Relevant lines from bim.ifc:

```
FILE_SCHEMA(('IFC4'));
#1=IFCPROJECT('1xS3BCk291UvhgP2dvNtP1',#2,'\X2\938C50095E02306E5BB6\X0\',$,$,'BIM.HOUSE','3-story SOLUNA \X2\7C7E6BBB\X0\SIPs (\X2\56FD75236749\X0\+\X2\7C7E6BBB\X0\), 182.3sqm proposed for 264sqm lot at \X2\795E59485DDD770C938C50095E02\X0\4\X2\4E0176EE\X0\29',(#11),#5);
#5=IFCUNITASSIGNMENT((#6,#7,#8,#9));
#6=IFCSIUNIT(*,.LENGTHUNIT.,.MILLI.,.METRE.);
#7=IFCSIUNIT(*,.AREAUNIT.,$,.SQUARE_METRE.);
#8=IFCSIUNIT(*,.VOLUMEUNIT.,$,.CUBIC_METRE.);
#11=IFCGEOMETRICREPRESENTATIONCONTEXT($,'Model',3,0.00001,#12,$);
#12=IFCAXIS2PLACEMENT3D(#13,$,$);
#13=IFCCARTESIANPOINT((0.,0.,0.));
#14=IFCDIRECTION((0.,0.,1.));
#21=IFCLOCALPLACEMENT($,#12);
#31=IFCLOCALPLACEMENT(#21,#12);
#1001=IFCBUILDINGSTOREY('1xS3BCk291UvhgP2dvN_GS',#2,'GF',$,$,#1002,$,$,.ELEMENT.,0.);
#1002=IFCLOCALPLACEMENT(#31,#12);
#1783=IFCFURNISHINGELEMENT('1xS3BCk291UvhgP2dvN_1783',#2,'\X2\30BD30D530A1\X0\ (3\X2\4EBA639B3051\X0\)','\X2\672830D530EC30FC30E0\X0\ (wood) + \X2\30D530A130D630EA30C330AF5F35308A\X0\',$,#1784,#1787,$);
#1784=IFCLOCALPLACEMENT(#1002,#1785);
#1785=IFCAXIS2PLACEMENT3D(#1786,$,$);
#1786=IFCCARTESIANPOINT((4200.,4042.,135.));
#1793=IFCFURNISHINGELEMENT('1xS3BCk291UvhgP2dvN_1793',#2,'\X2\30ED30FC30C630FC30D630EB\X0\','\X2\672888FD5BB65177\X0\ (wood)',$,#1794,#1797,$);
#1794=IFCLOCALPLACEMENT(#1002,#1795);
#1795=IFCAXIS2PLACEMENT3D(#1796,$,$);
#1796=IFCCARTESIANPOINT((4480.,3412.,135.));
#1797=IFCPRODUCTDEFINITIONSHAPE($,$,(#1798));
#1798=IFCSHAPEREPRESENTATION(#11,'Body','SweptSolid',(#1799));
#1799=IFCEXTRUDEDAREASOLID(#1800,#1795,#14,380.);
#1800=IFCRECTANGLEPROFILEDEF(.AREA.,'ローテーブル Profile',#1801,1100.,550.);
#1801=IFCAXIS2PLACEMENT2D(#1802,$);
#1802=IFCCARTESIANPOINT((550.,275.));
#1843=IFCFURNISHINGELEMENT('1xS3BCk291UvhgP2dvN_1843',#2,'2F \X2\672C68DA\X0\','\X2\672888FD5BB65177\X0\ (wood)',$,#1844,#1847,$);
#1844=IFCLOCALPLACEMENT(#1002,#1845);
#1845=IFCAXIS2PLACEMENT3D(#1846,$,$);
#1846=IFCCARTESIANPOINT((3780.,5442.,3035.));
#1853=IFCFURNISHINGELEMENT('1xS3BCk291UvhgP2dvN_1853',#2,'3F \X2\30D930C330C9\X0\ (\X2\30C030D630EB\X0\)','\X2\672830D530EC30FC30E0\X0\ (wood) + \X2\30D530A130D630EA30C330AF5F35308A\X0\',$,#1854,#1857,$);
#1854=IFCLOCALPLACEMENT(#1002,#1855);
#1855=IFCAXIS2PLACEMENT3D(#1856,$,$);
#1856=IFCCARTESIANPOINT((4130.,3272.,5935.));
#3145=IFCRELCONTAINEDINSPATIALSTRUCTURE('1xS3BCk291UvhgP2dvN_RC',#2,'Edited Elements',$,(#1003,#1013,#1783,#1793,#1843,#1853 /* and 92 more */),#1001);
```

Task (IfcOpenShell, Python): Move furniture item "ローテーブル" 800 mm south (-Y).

```python
import ifcopenshell
import ifcopenshell.api.geometry
import ifcopenshell.util.placement
import ifcopenshell.util.unit

model = ifcopenshell.open("bim.ifc")
unit_scale = ifcopenshell.util.unit.calculate_unit_scale(model)

item = model.by_id(1793)
matrix = ifcopenshell.util.placement.get_local_placement(item.ObjectPlacement)
matrix[1, 3] -= 0.8 / unit_scale
ifcopenshell.api.geometry.edit_object_placement(model, product=item, matrix=matrix, is_si=False)

print(ifcopenshell.util.placement.get_local_placement(item.ObjectPlacement).round(3) + 0.0)

model.write("bim_updated.ifc")
```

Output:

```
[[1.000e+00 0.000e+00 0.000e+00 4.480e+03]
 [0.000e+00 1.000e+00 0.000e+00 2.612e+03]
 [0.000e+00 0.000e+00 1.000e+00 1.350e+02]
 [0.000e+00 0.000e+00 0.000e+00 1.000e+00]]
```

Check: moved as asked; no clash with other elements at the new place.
